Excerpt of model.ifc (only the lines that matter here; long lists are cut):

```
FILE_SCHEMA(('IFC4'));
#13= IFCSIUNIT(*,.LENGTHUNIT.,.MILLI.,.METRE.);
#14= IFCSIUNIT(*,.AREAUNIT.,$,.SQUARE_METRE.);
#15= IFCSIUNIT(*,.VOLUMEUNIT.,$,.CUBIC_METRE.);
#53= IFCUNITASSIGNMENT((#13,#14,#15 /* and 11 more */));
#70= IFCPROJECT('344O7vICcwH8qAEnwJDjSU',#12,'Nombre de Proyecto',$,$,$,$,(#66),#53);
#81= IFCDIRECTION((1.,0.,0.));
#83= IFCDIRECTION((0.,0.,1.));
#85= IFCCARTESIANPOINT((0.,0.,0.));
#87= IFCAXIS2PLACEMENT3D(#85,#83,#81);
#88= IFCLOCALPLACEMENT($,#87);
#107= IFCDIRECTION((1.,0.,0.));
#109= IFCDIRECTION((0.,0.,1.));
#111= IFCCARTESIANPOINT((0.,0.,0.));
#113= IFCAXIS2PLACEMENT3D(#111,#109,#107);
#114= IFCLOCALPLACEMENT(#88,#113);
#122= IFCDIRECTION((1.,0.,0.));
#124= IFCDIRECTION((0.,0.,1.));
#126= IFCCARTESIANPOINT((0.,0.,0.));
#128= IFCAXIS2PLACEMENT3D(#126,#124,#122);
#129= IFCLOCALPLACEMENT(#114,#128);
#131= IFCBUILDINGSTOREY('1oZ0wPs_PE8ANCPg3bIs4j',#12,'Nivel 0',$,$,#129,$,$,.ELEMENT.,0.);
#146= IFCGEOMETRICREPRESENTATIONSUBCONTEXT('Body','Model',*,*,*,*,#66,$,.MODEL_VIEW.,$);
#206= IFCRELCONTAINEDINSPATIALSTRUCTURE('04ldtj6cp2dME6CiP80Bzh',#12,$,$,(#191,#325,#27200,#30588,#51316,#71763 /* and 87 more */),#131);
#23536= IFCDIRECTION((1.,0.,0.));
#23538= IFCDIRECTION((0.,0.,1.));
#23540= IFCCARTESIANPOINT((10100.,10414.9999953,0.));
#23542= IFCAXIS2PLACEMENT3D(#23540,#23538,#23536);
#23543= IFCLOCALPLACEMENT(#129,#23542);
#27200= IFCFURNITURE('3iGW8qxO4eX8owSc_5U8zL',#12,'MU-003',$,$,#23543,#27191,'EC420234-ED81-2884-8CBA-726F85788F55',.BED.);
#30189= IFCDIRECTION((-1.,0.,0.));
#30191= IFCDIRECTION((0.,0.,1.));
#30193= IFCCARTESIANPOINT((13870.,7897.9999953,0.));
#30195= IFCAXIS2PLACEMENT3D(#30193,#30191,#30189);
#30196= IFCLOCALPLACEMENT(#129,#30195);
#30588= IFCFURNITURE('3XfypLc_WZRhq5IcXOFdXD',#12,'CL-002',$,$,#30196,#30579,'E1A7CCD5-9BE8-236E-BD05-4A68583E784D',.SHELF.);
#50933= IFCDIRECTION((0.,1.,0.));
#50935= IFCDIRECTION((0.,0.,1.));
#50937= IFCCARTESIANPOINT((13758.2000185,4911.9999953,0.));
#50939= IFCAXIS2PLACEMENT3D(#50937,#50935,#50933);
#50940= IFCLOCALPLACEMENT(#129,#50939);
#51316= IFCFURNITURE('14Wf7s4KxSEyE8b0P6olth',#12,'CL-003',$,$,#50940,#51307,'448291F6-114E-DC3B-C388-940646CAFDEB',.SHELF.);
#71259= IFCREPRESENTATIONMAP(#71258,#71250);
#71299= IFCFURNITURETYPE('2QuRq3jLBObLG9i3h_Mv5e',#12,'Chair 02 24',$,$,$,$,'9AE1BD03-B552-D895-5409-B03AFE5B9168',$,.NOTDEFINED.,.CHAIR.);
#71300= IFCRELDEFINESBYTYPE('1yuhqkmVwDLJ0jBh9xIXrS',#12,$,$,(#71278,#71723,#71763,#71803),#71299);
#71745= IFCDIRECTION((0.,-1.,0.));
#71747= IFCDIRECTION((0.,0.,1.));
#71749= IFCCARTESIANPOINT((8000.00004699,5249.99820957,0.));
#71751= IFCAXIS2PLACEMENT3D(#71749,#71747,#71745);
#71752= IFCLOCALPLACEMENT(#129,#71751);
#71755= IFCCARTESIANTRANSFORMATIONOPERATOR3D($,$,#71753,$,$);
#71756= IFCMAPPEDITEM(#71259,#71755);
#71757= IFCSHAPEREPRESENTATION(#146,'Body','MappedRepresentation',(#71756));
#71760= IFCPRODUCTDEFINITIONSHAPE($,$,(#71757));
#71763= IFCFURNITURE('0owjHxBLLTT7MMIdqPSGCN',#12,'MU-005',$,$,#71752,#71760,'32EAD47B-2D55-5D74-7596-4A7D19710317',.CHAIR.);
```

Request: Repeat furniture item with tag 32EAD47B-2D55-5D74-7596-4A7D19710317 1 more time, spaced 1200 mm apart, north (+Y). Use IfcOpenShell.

```python
import numpy as np
import ifcopenshell
import ifcopenshell.api.geometry
import ifcopenshell.api.root
import ifcopenshell.util.element
import ifcopenshell.util.placement
import ifcopenshell.util.unit

model = ifcopenshell.open("model.ifc")
unit_scale = ifcopenshell.util.unit.calculate_unit_scale(model)


def reuse_history(source, copy):
    """copy_class also copies each property set's owner history, people and application; keep the originals."""
    for rel in copy.IsDefinedBy:
        if rel.is_a("IfcRelDefinesByProperties") and (history := rel.RelatingPropertyDefinition.OwnerHistory):
            rel.RelatingPropertyDefinition.OwnerHistory = source.OwnerHistory
            ifcopenshell.util.element.remove_deep2(model, history)


source = model.by_guid("0owjHxBLLTT7MMIdqPSGCN")
base = ifcopenshell.util.placement.get_local_placement(source.ObjectPlacement)
step = np.array([0.0, 1.0, 0.0]) * 1.2 / unit_scale

for i in range(1, 2):
    copy = ifcopenshell.api.root.copy_class(model, product=source)
    copy.Representation = ifcopenshell.util.element.copy_deep(
        model, source.Representation, exclude=["IfcGeometricRepresentationContext", "IfcRepresentationMap"]
    )
    copy.Tag = None
    reuse_history(source, copy)
    matrix = base.copy()
    matrix[:3, 3] += i * step
    print("added at", matrix[:3, 3].round(3) + 0.0)
    ifcopenshell.api.geometry.edit_object_placement(model, product=copy, matrix=matrix, is_si=False)

model.write("model_v2.ifc")
```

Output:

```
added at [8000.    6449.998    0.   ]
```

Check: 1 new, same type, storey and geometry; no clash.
